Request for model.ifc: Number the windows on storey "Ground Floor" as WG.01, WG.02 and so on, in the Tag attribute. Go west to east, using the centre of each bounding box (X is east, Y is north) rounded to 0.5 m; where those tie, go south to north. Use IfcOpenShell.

First a look at what the model holds.

```python
import ifcopenshell
import ifcopenshell.util.element
import ifcopenshell.util.placement

model = ifcopenshell.open("model.ifc")
print(model.schema)
storey = next(s for s in model.by_type("IfcBuildingStorey") if s.Name == "Ground Floor")
windows = [e for e in ifcopenshell.util.element.get_decomposition(storey) if e.is_a("IfcWindow")]
for e in sorted(windows, key=lambda e: e.id()):
    origin = ifcopenshell.util.placement.get_local_placement(e.ObjectPlacement)[:3, 3]
    print(e.id(), e.Tag, e.Name, origin.round(2) + 0.0, sep=" | ")
```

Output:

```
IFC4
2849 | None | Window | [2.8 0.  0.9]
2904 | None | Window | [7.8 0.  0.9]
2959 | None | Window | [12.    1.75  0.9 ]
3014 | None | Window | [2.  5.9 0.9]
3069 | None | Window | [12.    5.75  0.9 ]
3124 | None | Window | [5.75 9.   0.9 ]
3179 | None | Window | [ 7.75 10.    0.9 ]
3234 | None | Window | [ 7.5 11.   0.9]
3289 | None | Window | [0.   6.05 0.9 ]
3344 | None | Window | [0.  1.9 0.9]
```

```python
import ifcopenshell
import ifcopenshell.geom
import ifcopenshell.util.element
import ifcopenshell.util.shape

model = ifcopenshell.open("model.ifc")
settings = ifcopenshell.geom.settings()
settings.set("use-world-coords", True)


def centre(element):
    shape = ifcopenshell.geom.create_shape(settings, element)
    return ifcopenshell.util.shape.get_bbox_centroid(shape.geometry)


storey = next(s for s in model.by_type("IfcBuildingStorey") if s.Name == "Ground Floor")
windows = [e for e in ifcopenshell.util.element.get_decomposition(storey) if e.is_a("IfcWindow")]

# Insertion points can sit at a corner or the storey origin, so sort by the geometry (in metres).
centres = {e: centre(e) for e in windows}
windows.sort(key=lambda e: (round(centres[e][0] / 0.5), centres[e][1]))

for i, e in enumerate(windows, start=1):
    number = f"WG.{i:02d}"
    e.Tag = number
    print(e.id(), number)

model.write("model_rev.ifc")
```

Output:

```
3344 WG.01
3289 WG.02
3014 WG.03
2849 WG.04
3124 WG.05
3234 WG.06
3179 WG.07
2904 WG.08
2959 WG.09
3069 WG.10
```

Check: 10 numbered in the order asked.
